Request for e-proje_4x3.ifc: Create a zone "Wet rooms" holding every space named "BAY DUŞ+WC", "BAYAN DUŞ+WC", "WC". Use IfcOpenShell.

First a look at what the model holds.

```python
import ifcopenshell

model = ifcopenshell.open("e-proje_4x3.ifc")
print(model.schema)
seen = {}
for space in model.by_type("IfcSpace"):
    seen[space.LongName] = seen.get(space.LongName, 0) + 1
for name, count in sorted(seen.items(), key=str):
    print(count, "x", name)
print("zones:", [z.Name for z in model.by_type("IfcZone")][:20])
```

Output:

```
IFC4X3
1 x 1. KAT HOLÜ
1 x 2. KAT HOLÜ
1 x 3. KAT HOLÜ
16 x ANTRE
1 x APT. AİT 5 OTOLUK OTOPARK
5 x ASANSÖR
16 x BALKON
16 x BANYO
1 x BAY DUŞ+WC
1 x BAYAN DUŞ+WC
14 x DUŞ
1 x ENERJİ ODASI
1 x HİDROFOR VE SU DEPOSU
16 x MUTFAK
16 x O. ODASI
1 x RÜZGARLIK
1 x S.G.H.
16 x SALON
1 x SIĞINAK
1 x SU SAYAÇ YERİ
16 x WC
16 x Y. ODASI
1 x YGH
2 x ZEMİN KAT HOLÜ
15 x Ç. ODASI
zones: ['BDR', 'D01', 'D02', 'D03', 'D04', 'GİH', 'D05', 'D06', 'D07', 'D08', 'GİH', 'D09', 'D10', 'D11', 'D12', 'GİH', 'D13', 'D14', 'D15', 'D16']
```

```python
import ifcopenshell
import ifcopenshell.api.group
import ifcopenshell.api.root

model = ifcopenshell.open("e-proje_4x3.ifc")

names = {"BAY DUŞ+WC", "BAYAN DUŞ+WC", "WC"}
spaces = [s for s in model.by_type("IfcSpace") if s.LongName in names]

zone = ifcopenshell.api.root.create_entity(model, ifc_class="IfcZone", name="Wet rooms")
ifcopenshell.api.group.assign_group(model, products=spaces, group=zone)
print(len(spaces), "spaces in", zone.Name)

model.write("e-proje_4x3_rev.ifc")
```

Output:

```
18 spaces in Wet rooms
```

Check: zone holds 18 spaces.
